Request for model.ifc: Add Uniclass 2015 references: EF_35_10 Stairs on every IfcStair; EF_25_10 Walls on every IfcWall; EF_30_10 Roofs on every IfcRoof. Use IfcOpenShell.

First a look at what the model holds.

```python
import ifcopenshell

model = ifcopenshell.open("model.ifc")
print(model.schema)
print("classifications:", [c.Name for c in model.by_type("IfcClassification")])
for ifc_class in ("IfcDoor", "IfcRoof", "IfcStair", "IfcWall", "IfcWindow"):
    print(ifc_class, len(model.by_type(ifc_class)))
```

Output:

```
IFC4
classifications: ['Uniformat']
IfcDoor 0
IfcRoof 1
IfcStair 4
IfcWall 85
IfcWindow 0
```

```python
import ifcopenshell
import ifcopenshell.api.classification

model = ifcopenshell.open("model.ifc")

system = ifcopenshell.api.classification.add_classification(model, classification="Uniclass 2015")

codes = {
    "IfcStair": ("EF_35_10", "Stairs"),
    "IfcWall": ("EF_25_10", "Walls"),
    "IfcRoof": ("EF_30_10", "Roofs"),
}
for ifc_class, (code, name) in codes.items():
    products = model.by_type(ifc_class)
    ifcopenshell.api.classification.add_reference(
        model, products=products, classification=system, identification=code, name=name
    )
    print(code, len(products))

model.write("model_v2.ifc")
```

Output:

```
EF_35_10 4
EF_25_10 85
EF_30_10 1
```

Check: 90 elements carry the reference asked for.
